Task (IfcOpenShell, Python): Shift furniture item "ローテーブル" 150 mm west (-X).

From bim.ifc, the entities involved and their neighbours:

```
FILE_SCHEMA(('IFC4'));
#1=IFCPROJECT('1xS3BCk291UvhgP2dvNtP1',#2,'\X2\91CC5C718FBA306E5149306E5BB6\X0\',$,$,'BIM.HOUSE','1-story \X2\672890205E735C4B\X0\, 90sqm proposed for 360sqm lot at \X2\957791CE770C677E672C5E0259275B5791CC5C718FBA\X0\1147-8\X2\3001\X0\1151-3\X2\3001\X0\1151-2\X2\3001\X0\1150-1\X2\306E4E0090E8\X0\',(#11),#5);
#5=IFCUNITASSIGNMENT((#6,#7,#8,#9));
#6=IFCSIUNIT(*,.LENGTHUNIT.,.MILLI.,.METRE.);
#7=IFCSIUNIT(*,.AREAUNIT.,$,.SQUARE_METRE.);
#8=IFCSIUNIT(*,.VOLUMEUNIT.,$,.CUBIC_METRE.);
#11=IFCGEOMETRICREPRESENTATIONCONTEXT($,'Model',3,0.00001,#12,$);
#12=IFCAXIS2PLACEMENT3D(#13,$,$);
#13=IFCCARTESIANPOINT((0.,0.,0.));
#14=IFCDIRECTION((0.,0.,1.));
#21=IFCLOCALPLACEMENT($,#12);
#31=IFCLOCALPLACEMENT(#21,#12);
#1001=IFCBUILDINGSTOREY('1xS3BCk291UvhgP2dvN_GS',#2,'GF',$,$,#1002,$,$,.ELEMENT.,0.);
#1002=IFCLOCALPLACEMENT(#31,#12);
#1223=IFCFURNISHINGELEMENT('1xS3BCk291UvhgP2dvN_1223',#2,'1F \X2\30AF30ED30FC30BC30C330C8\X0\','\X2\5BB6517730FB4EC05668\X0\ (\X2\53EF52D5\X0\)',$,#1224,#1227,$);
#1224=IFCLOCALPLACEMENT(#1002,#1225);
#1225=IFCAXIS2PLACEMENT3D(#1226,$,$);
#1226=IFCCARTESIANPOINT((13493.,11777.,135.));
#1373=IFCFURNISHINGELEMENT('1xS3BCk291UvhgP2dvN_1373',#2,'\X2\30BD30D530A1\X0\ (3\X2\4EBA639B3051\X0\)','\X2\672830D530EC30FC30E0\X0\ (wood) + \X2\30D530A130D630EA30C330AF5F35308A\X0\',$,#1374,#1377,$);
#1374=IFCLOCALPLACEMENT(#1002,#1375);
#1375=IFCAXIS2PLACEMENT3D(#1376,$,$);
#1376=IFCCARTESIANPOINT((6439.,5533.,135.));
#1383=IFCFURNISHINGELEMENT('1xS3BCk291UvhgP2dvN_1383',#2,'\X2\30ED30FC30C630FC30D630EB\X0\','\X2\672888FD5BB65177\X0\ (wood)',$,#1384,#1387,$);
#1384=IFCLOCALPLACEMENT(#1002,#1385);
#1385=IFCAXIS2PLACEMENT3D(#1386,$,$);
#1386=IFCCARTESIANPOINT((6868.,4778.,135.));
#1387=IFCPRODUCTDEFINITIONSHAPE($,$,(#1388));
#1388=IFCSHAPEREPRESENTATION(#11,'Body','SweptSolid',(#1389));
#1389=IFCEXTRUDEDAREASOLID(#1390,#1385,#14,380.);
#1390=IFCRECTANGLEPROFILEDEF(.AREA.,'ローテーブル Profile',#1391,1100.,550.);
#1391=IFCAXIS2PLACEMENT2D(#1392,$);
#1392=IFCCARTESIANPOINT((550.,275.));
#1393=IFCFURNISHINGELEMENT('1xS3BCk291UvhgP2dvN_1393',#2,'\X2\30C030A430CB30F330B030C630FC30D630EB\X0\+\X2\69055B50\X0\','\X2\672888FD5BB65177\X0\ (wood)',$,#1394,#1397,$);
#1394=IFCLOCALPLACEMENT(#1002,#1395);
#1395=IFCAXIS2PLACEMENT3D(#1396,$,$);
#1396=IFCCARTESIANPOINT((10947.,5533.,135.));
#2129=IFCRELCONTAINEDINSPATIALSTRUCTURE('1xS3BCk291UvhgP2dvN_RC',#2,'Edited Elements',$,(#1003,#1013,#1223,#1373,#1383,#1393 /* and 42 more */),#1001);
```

```python
import ifcopenshell
import ifcopenshell.api.geometry
import ifcopenshell.util.placement
import ifcopenshell.util.unit

model = ifcopenshell.open("bim.ifc")
unit_scale = ifcopenshell.util.unit.calculate_unit_scale(model)

item = model.by_guid("1xS3BCk291UvhgP2dvN_1383")
matrix = ifcopenshell.util.placement.get_local_placement(item.ObjectPlacement)
matrix[0, 3] -= 0.15 / unit_scale
ifcopenshell.api.geometry.edit_object_placement(model, product=item, matrix=matrix, is_si=False)

print(ifcopenshell.util.placement.get_local_placement(item.ObjectPlacement).round(3) + 0.0)

model.write("bim_v2.ifc")
```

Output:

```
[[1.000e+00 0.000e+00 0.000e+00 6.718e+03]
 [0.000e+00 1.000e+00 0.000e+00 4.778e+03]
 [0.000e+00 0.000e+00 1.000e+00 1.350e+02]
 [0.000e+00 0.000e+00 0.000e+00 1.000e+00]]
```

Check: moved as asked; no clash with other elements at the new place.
